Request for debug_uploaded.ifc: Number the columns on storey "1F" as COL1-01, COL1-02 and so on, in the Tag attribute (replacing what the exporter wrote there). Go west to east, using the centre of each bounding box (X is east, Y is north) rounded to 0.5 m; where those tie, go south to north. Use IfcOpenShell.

First a look at what the model holds.

```python
import ifcopenshell
import ifcopenshell.util.element
import ifcopenshell.util.placement

model = ifcopenshell.open("debug_uploaded.ifc")
print(model.schema)
storey = next(s for s in model.by_type("IfcBuildingStorey") if s.Name == "1F")
columns = [e for e in ifcopenshell.util.element.get_decomposition(storey) if e.is_a("IfcColumn")]
for e in sorted(columns, key=lambda e: e.id()):
    origin = ifcopenshell.util.placement.get_local_placement(e.ObjectPlacement)[:3, 3]
    print(e.id(), e.Tag, e.Name, origin.round(2) + 0.0, sep=" | ")
```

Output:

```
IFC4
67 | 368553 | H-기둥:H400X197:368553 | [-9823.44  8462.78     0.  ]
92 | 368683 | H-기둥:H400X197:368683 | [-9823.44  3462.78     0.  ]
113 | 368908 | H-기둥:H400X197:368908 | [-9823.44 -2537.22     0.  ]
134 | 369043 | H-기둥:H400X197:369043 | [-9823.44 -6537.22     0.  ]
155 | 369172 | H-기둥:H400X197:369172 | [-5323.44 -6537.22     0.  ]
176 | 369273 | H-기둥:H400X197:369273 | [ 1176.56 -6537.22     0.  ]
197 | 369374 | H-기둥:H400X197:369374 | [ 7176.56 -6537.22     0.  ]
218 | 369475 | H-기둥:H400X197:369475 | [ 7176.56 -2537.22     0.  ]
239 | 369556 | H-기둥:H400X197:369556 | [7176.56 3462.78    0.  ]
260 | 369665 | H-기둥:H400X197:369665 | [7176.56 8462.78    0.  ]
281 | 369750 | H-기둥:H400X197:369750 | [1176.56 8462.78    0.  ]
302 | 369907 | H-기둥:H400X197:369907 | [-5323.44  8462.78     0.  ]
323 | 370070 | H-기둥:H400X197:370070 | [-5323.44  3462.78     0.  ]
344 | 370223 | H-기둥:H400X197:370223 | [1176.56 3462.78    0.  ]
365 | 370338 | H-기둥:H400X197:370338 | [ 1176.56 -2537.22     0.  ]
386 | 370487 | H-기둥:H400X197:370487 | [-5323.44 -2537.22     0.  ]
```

```python
import ifcopenshell
import ifcopenshell.geom
import ifcopenshell.util.element
import ifcopenshell.util.shape

model = ifcopenshell.open("debug_uploaded.ifc")
settings = ifcopenshell.geom.settings()
settings.set("use-world-coords", True)


def centre(element):
    shape = ifcopenshell.geom.create_shape(settings, element)
    return ifcopenshell.util.shape.get_bbox_centroid(shape.geometry)


storey = next(s for s in model.by_type("IfcBuildingStorey") if s.Name == "1F")
columns = [e for e in ifcopenshell.util.element.get_decomposition(storey) if e.is_a("IfcColumn")]

# Insertion points can sit at a corner or the storey origin, so sort by the geometry (in metres).
centres = {e: centre(e) for e in columns}
columns.sort(key=lambda e: (round(centres[e][0] / 0.5), centres[e][1]))

for i, e in enumerate(columns, start=1):
    number = f"COL1-{i:02d}"
    e.Tag = number
    print(e.id(), number)

model.write("debug_uploaded_updated.ifc")
```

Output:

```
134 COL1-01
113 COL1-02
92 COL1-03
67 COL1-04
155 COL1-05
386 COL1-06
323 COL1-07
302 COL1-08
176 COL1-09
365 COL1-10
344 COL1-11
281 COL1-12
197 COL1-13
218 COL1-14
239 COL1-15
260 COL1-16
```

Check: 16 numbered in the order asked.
